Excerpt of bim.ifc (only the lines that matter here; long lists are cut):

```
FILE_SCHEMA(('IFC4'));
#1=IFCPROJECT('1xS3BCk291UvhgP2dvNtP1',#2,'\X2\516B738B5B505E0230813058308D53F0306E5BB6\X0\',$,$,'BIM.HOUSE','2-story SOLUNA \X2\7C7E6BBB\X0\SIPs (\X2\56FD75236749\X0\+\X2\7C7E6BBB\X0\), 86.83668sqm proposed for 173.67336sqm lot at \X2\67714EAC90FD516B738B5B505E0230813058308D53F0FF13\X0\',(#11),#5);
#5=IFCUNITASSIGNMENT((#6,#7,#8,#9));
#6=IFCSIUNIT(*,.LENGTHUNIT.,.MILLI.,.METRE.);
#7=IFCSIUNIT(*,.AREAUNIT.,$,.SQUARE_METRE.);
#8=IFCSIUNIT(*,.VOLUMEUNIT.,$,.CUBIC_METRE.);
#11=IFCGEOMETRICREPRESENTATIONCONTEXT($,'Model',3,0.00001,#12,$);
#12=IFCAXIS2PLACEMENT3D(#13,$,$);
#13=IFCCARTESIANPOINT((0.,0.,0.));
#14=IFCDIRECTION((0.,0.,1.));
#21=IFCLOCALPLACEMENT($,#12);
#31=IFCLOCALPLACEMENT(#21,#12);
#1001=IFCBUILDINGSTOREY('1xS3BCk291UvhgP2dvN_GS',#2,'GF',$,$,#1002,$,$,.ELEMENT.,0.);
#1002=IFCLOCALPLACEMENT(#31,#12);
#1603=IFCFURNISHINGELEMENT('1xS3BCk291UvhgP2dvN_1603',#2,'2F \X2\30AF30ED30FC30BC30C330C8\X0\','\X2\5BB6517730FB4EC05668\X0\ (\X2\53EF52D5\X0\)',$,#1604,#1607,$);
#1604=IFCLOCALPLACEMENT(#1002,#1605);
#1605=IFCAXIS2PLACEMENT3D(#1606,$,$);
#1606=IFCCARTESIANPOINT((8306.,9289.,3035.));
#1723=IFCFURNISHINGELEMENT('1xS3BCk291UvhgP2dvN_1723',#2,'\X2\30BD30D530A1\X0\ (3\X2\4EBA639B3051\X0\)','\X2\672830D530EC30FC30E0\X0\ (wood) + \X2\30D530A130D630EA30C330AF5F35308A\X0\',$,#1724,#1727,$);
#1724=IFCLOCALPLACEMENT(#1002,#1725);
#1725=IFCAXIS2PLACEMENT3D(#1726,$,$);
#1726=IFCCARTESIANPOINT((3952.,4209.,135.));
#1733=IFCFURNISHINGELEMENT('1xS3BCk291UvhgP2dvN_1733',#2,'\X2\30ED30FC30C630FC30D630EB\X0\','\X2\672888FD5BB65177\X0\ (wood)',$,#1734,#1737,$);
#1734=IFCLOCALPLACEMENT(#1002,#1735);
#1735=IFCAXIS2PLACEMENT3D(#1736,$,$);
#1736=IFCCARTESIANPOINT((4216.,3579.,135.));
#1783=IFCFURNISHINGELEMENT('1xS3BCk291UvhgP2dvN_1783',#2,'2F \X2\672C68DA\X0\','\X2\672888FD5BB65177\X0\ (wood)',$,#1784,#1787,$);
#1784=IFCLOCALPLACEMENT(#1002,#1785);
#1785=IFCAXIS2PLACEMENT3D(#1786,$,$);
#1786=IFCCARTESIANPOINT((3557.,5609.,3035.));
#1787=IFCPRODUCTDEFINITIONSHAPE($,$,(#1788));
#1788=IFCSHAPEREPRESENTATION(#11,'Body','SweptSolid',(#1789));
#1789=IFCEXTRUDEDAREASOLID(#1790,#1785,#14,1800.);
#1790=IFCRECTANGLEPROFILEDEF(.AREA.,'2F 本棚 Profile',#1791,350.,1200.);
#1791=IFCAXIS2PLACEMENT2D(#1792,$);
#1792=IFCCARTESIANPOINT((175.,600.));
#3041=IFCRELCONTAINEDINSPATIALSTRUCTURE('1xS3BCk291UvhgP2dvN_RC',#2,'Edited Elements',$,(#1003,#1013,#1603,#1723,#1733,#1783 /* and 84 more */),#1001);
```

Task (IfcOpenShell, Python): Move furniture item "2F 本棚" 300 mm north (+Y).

```python
import ifcopenshell
import ifcopenshell.api.geometry
import ifcopenshell.util.placement
import ifcopenshell.util.unit

model = ifcopenshell.open("bim.ifc")
unit_scale = ifcopenshell.util.unit.calculate_unit_scale(model)

item = model.by_id(1783)
matrix = ifcopenshell.util.placement.get_local_placement(item.ObjectPlacement)
matrix[1, 3] += 0.3 / unit_scale
ifcopenshell.api.geometry.edit_object_placement(model, product=item, matrix=matrix, is_si=False)

print(ifcopenshell.util.placement.get_local_placement(item.ObjectPlacement).round(3) + 0.0)

model.write("bim_updated.ifc")
```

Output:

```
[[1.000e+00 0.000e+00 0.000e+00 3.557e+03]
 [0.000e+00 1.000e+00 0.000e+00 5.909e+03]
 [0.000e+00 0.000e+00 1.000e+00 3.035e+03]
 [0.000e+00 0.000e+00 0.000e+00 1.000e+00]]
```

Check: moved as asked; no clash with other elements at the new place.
